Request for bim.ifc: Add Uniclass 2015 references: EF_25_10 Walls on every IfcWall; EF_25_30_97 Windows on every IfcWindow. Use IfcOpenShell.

First a look at what the model holds.

```python
import ifcopenshell

model = ifcopenshell.open("bim.ifc")
print(model.schema)
print("classifications:", [c.Name for c in model.by_type("IfcClassification")])
for ifc_class in ("IfcDoor", "IfcRoof", "IfcStair", "IfcWall", "IfcWindow"):
    print(ifc_class, len(model.by_type(ifc_class)))
```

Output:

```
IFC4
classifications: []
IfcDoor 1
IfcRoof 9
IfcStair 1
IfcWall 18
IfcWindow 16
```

```python
import ifcopenshell
import ifcopenshell.api.classification

model = ifcopenshell.open("bim.ifc")

system = ifcopenshell.api.classification.add_classification(model, classification="Uniclass 2015")

codes = {
    "IfcWall": ("EF_25_10", "Walls"),
    "IfcWindow": ("EF_25_30_97", "Windows"),
}
for ifc_class, (code, name) in codes.items():
    products = model.by_type(ifc_class)
    ifcopenshell.api.classification.add_reference(
        model, products=products, classification=system, identification=code, name=name
    )
    print(code, len(products))

model.write("bim-out.ifc")
```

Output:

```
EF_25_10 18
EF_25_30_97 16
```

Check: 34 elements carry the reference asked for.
